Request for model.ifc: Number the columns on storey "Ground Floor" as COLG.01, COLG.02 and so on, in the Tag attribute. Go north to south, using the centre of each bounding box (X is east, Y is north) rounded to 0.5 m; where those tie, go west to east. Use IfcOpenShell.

First a look at what the model holds.

```python
import ifcopenshell
import ifcopenshell.util.element
import ifcopenshell.util.placement

model = ifcopenshell.open("model.ifc")
print(model.schema)
storey = next(s for s in model.by_type("IfcBuildingStorey") if s.Name == "Ground Floor")
columns = [e for e in ifcopenshell.util.element.get_decomposition(storey) if e.is_a("IfcColumn")]
for e in sorted(columns, key=lambda e: e.id()):
    origin = ifcopenshell.util.placement.get_local_placement(e.ObjectPlacement)[:3, 3]
    print(e.id(), e.Tag, e.Name, origin.round(2) + 0.0, sep=" | ")
```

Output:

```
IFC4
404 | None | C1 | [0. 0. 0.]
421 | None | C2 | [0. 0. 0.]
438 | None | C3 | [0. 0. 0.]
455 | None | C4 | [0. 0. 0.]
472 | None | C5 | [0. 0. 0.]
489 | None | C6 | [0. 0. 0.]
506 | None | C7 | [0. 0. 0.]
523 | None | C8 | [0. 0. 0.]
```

```python
import ifcopenshell
import ifcopenshell.geom
import ifcopenshell.util.element
import ifcopenshell.util.shape

model = ifcopenshell.open("model.ifc")
settings = ifcopenshell.geom.settings()
settings.set("use-world-coords", True)


def centre(element):
    shape = ifcopenshell.geom.create_shape(settings, element)
    return ifcopenshell.util.shape.get_bbox_centroid(shape.geometry)


storey = next(s for s in model.by_type("IfcBuildingStorey") if s.Name == "Ground Floor")
columns = [e for e in ifcopenshell.util.element.get_decomposition(storey) if e.is_a("IfcColumn")]

# Insertion points can sit at a corner or the storey origin, so sort by the geometry (in metres).
centres = {e: centre(e) for e in columns}
columns.sort(key=lambda e: (-round(centres[e][1] / 0.5), centres[e][0]))

for i, e in enumerate(columns, start=1):
    number = f"COLG.{i:02d}"
    e.Tag = number
    print(e.id(), number)

model.write("model-out.ifc")
```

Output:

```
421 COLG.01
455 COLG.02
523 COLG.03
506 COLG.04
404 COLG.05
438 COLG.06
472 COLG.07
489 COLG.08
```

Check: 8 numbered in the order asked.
